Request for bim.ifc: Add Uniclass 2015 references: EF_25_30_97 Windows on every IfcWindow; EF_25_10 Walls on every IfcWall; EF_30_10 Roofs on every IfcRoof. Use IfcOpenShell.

First a look at what the model holds.

```python
import ifcopenshell

model = ifcopenshell.open("bim.ifc")
print(model.schema)
print("classifications:", [c.Name for c in model.by_type("IfcClassification")])
for ifc_class in ("IfcDoor", "IfcRoof", "IfcStair", "IfcWall", "IfcWindow"):
    print(ifc_class, len(model.by_type(ifc_class)))
```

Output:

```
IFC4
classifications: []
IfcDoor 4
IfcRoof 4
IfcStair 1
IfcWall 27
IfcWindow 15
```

```python
import ifcopenshell
import ifcopenshell.api.classification

model = ifcopenshell.open("bim.ifc")

system = ifcopenshell.api.classification.add_classification(model, classification="Uniclass 2015")

codes = {
    "IfcWindow": ("EF_25_30_97", "Windows"),
    "IfcWall": ("EF_25_10", "Walls"),
    "IfcRoof": ("EF_30_10", "Roofs"),
}
for ifc_class, (code, name) in codes.items():
    products = model.by_type(ifc_class)
    ifcopenshell.api.classification.add_reference(
        model, products=products, classification=system, identification=code, name=name
    )
    print(code, len(products))

model.write("bim_updated.ifc")
```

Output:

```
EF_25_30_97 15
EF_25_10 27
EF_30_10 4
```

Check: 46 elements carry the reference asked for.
